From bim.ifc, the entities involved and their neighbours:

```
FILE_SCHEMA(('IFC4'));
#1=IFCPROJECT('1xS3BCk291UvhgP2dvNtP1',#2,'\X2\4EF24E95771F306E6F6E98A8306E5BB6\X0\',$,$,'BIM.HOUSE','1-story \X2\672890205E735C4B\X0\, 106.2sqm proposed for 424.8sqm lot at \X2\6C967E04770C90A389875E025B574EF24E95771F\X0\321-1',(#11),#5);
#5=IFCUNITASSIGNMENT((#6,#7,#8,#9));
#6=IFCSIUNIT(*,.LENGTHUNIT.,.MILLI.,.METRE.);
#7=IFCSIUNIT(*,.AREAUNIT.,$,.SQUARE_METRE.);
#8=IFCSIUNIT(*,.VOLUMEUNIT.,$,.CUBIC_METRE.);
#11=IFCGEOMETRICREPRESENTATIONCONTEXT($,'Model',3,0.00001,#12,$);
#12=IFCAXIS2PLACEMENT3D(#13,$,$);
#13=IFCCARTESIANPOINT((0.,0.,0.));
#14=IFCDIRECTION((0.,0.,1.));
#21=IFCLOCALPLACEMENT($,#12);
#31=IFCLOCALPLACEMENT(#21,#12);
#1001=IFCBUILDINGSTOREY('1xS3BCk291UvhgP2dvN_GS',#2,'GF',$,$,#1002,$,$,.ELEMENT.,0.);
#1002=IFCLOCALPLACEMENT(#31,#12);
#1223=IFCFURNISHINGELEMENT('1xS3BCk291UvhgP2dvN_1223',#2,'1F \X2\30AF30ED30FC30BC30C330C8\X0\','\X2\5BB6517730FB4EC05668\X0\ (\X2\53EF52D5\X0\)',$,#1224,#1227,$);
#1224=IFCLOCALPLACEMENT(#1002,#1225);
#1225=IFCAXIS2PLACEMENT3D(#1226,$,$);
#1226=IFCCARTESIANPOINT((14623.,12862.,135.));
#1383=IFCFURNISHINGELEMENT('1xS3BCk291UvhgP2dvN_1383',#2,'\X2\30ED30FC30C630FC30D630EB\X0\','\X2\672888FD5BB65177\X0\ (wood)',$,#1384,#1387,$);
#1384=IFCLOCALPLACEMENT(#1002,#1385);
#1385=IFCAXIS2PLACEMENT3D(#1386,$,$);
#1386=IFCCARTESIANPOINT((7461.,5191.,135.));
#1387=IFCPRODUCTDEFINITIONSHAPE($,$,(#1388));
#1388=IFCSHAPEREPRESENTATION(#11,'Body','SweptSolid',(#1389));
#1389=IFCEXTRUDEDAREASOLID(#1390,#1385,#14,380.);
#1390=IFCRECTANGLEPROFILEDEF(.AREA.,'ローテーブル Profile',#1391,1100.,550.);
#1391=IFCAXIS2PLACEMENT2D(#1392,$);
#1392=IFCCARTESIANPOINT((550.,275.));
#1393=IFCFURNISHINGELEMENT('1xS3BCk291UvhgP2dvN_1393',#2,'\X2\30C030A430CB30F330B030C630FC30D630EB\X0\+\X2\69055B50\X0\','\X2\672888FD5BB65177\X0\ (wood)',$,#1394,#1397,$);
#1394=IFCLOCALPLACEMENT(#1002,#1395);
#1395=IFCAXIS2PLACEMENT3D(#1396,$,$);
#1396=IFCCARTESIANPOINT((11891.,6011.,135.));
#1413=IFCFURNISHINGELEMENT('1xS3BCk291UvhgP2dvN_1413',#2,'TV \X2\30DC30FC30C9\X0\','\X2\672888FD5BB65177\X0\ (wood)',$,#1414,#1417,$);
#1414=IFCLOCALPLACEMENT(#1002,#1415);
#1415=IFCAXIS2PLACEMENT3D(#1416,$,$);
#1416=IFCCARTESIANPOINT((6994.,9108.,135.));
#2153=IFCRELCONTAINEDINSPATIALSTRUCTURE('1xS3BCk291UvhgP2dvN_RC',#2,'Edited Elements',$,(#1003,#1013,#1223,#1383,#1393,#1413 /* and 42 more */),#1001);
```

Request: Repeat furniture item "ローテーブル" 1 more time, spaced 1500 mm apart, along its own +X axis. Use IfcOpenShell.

```python
import ifcopenshell
import ifcopenshell.api.geometry
import ifcopenshell.api.root
import ifcopenshell.util.element
import ifcopenshell.util.placement

model = ifcopenshell.open("bim.ifc")


def reuse_history(source, copy):
    """copy_class also copies each property set's owner history, people and application; keep the originals."""
    for rel in copy.IsDefinedBy:
        if rel.is_a("IfcRelDefinesByProperties") and (history := rel.RelatingPropertyDefinition.OwnerHistory):
            rel.RelatingPropertyDefinition.OwnerHistory = source.OwnerHistory
            ifcopenshell.util.element.remove_deep2(model, history)


source = model.by_guid("1xS3BCk291UvhgP2dvN_1383")
base = ifcopenshell.util.placement.get_local_placement(source.ObjectPlacement)
step = base[:3, 0] * 1500.0

for i in range(1, 2):
    copy = ifcopenshell.api.root.copy_class(model, product=source)
    copy.Representation = ifcopenshell.util.element.copy_deep(
        model, source.Representation, exclude=["IfcGeometricRepresentationContext", "IfcRepresentationMap"]
    )
    reuse_history(source, copy)
    matrix = base.copy()
    matrix[:3, 3] += i * step
    print("added at", matrix[:3, 3].round(3) + 0.0)
    ifcopenshell.api.geometry.edit_object_placement(model, product=copy, matrix=matrix, is_si=False)

model.write("bim-out.ifc")
```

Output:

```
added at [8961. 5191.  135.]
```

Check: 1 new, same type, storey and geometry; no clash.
